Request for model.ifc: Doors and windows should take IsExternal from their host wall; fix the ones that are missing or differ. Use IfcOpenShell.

First a look at what the model holds.

```python
import ifcopenshell
import ifcopenshell.util.element

model = ifcopenshell.open("model.ifc")
print(model.schema)
seen = {}
for e in model.by_type("IfcDoor") + model.by_type("IfcWindow"):
    if not e.FillsVoids:
        continue
    host = e.FillsVoids[0].RelatingOpeningElement.VoidsElements[0].RelatingBuildingElement
    own = ifcopenshell.util.element.get_pset(e, f"Pset_{e.is_a()[3:].removesuffix('StandardCase')}Common", "IsExternal")
    wall = ifcopenshell.util.element.get_pset(host, "Pset_WallCommon", "IsExternal")
    seen[e.is_a(), own, wall] = seen.get((e.is_a(), own, wall), 0) + 1
for (cls, own, wall), count in sorted(seen.items(), key=str):
    print(count, cls, "IsExternal:", own, "| host wall:", wall)
```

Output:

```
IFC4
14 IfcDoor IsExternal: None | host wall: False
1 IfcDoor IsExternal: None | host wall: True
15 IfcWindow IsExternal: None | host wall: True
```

```python
import ifcopenshell
import ifcopenshell.api.pset
import ifcopenshell.util.element

model = ifcopenshell.open("model.ifc")

count = 0
for ifc_class, pset_name in (("IfcDoor", "Pset_DoorCommon"), ("IfcWindow", "Pset_WindowCommon")):
    for e in model.by_type(ifc_class):
        if not e.FillsVoids:
            continue
        host = e.FillsVoids[0].RelatingOpeningElement.VoidsElements[0].RelatingBuildingElement
        external = ifcopenshell.util.element.get_pset(host, "Pset_WallCommon", "IsExternal")
        if external is None or ifcopenshell.util.element.get_pset(e, pset_name, "IsExternal") == external:
            continue
        pset = ifcopenshell.api.pset.add_pset(model, product=e, name=pset_name)
        ifcopenshell.api.pset.edit_pset(model, pset=pset, properties={"IsExternal": external})
        count += 1

print(count, "updated")

model.write("model_rev.ifc")
```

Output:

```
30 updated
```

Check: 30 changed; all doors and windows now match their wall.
